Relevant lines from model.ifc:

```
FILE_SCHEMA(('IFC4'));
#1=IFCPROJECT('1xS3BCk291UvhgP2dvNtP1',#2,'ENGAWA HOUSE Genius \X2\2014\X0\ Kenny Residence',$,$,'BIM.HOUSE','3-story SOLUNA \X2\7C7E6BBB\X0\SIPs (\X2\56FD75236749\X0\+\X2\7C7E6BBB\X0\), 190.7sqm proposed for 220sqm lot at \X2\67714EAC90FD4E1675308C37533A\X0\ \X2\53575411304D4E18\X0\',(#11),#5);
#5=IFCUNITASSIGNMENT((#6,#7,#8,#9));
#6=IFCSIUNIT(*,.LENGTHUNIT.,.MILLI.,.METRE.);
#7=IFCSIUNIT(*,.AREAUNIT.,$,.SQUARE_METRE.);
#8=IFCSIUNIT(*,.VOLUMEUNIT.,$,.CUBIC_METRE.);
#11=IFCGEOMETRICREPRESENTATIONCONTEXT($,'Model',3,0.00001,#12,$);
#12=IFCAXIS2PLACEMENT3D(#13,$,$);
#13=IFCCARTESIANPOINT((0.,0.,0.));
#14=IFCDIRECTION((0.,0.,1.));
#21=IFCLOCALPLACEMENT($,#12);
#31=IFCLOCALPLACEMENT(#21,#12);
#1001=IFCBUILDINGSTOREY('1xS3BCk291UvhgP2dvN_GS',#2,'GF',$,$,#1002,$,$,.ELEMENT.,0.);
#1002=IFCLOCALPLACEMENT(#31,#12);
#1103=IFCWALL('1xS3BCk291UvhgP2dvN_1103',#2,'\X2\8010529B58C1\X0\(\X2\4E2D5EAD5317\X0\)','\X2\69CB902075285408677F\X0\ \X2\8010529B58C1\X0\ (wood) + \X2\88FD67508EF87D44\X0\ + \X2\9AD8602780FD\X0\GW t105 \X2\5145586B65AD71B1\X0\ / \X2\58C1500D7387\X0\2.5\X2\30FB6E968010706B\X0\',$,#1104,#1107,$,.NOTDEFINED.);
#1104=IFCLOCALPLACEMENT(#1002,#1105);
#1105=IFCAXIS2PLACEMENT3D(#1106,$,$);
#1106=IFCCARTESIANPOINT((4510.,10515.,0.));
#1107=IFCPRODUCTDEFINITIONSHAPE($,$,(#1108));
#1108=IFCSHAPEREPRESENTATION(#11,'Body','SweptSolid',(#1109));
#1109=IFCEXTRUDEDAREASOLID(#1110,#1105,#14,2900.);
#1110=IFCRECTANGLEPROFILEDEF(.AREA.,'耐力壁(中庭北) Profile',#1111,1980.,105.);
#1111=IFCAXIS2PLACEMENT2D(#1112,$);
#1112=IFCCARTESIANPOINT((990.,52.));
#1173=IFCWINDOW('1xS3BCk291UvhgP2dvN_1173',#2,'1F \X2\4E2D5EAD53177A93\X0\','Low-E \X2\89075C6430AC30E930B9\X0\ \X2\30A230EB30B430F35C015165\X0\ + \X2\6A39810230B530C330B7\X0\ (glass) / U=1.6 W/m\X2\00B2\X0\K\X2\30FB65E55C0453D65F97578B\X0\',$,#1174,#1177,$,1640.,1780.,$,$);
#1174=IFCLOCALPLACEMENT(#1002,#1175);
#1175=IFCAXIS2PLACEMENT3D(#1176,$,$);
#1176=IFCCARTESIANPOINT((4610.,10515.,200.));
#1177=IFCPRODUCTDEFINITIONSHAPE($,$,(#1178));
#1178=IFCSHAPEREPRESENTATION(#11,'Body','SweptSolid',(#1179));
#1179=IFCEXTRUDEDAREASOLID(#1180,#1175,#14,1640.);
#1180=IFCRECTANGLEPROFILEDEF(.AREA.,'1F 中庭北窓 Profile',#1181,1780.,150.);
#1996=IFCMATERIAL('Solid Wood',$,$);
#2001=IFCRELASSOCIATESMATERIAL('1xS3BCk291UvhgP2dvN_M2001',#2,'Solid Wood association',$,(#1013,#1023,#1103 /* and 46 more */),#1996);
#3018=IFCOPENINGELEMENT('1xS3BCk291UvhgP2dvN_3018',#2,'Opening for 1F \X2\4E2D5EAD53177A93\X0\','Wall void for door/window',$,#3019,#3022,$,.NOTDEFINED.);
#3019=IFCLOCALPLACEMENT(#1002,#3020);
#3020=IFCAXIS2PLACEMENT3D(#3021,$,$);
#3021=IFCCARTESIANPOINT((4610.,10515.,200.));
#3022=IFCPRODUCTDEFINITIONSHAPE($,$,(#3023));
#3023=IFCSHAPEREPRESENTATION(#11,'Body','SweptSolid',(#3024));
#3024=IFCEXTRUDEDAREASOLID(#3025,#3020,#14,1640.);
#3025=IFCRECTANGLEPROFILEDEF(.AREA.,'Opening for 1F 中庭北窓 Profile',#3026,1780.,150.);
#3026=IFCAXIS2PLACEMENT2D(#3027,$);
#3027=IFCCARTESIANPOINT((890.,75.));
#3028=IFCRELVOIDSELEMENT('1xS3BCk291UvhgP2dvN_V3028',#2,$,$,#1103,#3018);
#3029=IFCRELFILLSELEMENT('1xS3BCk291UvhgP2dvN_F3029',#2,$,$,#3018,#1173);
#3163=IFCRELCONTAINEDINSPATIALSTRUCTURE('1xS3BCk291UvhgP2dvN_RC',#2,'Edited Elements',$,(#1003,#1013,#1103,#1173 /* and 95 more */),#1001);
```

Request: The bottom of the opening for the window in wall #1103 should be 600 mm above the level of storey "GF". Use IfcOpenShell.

```python
import numpy as np
import ifcopenshell
import ifcopenshell.api.geometry
import ifcopenshell.geom
import ifcopenshell.util.element
import ifcopenshell.util.placement
import ifcopenshell.util.shape
import ifcopenshell.util.unit

model = ifcopenshell.open("model.ifc")
unit_scale = ifcopenshell.util.unit.calculate_unit_scale(model)

window = model.by_guid("1xS3BCk291UvhgP2dvN_1173")
opening = window.FillsVoids[0].RelatingOpeningElement
storey = ifcopenshell.util.element.get_container(window, ifc_class="IfcBuildingStorey")
level = ifcopenshell.util.placement.get_local_placement(storey.ObjectPlacement)[2, 3]

# The opening's origin need not be at the sill, so measure its lowest point.
shape = ifcopenshell.geom.create_shape(ifcopenshell.geom.settings(), opening)
bottom = ifcopenshell.util.shape.get_shape_bottom_elevation(shape, shape.geometry) / unit_scale
dz = level + 0.6 / unit_scale - bottom

shift = np.array([0.0, 0.0, dz])
# The window is not placed relative to its opening, so move both.
for product in (opening, window):
    matrix = ifcopenshell.util.placement.get_local_placement(product.ObjectPlacement)
    matrix[:3, 3] += shift
    ifcopenshell.api.geometry.edit_object_placement(model, product=product, matrix=matrix, is_si=False)

print(f"moved by {dz * unit_scale:+.3f} m")

model.write("model-out.ifc")
```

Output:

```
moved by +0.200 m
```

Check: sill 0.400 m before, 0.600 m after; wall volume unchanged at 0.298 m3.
